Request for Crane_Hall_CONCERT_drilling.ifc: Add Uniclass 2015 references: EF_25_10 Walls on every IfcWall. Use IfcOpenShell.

First a look at what the model holds.

```python
import ifcopenshell

model = ifcopenshell.open("Crane_Hall_CONCERT_drilling.ifc")
print(model.schema)
print("classifications:", [c.Name for c in model.by_type("IfcClassification")])
for ifc_class in ("IfcDoor", "IfcRoof", "IfcStair", "IfcWall", "IfcWindow"):
    print(ifc_class, len(model.by_type(ifc_class)))
```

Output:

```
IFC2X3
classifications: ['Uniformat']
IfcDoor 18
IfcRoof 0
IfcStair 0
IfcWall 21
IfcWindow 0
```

```python
import ifcopenshell
import ifcopenshell.api.classification

model = ifcopenshell.open("Crane_Hall_CONCERT_drilling.ifc")

# IFC2X3 requires Source and Edition and has no link from the project to the system.
system = model.create_entity("IfcClassification", Source="NBS", Edition="2015", Name="Uniclass 2015")

codes = {
    "IfcWall": ("EF_25_10", "Walls"),
}
for ifc_class, (code, name) in codes.items():
    products = model.by_type(ifc_class)
    ifcopenshell.api.classification.add_reference(
        model, products=products, classification=system, identification=code, name=name
    )
    print(code, len(products))

model.write("Crane_Hall_CONCERT_drilling_updated.ifc")
```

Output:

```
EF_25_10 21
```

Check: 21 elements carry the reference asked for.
